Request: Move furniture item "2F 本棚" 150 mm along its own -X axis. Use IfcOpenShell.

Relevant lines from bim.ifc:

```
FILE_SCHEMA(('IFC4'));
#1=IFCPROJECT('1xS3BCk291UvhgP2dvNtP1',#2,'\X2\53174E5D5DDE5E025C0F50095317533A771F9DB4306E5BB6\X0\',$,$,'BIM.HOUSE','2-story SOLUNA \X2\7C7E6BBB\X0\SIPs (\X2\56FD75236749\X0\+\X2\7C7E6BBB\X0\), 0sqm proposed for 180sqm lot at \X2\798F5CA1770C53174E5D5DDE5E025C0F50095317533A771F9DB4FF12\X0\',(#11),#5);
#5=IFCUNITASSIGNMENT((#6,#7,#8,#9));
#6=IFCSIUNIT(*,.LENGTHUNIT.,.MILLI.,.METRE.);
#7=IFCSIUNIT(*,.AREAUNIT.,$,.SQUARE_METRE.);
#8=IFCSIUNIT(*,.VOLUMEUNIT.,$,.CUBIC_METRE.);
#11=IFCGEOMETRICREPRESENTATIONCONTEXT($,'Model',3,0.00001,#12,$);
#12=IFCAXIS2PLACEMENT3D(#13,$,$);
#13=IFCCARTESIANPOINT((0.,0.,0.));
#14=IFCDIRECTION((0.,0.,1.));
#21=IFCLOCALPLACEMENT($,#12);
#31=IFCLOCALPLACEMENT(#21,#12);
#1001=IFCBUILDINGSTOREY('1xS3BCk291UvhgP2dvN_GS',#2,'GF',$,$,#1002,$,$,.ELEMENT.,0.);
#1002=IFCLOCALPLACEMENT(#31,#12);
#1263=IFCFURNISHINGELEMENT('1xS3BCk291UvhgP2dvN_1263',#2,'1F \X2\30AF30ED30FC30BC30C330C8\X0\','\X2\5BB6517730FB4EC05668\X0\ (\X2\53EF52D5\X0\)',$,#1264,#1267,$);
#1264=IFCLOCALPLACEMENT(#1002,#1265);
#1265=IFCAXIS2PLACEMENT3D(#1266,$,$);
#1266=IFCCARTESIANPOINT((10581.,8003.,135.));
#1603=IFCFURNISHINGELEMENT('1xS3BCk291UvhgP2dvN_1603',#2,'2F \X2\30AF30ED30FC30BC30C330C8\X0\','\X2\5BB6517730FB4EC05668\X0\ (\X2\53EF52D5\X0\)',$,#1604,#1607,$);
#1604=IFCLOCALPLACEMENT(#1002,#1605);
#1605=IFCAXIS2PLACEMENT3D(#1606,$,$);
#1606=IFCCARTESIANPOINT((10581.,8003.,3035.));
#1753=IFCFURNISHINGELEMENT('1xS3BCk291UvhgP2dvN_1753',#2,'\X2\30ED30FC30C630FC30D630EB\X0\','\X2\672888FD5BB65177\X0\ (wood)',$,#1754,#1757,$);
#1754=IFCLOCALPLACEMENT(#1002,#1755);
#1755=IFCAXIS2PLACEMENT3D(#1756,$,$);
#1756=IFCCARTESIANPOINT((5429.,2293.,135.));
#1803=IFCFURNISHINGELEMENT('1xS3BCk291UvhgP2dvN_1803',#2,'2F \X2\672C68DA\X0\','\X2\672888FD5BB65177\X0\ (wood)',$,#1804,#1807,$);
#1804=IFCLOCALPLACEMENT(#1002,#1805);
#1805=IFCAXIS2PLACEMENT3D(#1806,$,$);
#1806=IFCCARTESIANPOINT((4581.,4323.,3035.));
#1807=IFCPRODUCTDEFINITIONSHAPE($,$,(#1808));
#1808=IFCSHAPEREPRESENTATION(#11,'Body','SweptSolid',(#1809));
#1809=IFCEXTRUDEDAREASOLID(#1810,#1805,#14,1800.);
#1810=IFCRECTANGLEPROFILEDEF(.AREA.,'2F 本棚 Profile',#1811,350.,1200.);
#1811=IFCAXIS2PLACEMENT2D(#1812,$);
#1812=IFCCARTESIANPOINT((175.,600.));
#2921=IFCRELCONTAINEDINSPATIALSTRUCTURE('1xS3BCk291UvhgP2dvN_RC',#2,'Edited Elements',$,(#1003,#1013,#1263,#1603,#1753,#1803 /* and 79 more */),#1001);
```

```python
import ifcopenshell
import ifcopenshell.api.geometry
import ifcopenshell.util.placement
import ifcopenshell.util.unit

model = ifcopenshell.open("bim.ifc")
unit_scale = ifcopenshell.util.unit.calculate_unit_scale(model)

item = model.by_guid("1xS3BCk291UvhgP2dvN_1803")
matrix = ifcopenshell.util.placement.get_local_placement(item.ObjectPlacement)
matrix[:3, 3] -= matrix[:3, 0] * 0.15 / unit_scale
ifcopenshell.api.geometry.edit_object_placement(model, product=item, matrix=matrix, is_si=False)

print(ifcopenshell.util.placement.get_local_placement(item.ObjectPlacement).round(3) + 0.0)

model.write("bim-out.ifc")
```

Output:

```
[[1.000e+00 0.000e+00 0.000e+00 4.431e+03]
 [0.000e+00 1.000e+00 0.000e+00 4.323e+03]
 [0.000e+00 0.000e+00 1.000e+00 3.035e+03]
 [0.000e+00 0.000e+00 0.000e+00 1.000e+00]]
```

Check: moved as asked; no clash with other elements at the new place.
